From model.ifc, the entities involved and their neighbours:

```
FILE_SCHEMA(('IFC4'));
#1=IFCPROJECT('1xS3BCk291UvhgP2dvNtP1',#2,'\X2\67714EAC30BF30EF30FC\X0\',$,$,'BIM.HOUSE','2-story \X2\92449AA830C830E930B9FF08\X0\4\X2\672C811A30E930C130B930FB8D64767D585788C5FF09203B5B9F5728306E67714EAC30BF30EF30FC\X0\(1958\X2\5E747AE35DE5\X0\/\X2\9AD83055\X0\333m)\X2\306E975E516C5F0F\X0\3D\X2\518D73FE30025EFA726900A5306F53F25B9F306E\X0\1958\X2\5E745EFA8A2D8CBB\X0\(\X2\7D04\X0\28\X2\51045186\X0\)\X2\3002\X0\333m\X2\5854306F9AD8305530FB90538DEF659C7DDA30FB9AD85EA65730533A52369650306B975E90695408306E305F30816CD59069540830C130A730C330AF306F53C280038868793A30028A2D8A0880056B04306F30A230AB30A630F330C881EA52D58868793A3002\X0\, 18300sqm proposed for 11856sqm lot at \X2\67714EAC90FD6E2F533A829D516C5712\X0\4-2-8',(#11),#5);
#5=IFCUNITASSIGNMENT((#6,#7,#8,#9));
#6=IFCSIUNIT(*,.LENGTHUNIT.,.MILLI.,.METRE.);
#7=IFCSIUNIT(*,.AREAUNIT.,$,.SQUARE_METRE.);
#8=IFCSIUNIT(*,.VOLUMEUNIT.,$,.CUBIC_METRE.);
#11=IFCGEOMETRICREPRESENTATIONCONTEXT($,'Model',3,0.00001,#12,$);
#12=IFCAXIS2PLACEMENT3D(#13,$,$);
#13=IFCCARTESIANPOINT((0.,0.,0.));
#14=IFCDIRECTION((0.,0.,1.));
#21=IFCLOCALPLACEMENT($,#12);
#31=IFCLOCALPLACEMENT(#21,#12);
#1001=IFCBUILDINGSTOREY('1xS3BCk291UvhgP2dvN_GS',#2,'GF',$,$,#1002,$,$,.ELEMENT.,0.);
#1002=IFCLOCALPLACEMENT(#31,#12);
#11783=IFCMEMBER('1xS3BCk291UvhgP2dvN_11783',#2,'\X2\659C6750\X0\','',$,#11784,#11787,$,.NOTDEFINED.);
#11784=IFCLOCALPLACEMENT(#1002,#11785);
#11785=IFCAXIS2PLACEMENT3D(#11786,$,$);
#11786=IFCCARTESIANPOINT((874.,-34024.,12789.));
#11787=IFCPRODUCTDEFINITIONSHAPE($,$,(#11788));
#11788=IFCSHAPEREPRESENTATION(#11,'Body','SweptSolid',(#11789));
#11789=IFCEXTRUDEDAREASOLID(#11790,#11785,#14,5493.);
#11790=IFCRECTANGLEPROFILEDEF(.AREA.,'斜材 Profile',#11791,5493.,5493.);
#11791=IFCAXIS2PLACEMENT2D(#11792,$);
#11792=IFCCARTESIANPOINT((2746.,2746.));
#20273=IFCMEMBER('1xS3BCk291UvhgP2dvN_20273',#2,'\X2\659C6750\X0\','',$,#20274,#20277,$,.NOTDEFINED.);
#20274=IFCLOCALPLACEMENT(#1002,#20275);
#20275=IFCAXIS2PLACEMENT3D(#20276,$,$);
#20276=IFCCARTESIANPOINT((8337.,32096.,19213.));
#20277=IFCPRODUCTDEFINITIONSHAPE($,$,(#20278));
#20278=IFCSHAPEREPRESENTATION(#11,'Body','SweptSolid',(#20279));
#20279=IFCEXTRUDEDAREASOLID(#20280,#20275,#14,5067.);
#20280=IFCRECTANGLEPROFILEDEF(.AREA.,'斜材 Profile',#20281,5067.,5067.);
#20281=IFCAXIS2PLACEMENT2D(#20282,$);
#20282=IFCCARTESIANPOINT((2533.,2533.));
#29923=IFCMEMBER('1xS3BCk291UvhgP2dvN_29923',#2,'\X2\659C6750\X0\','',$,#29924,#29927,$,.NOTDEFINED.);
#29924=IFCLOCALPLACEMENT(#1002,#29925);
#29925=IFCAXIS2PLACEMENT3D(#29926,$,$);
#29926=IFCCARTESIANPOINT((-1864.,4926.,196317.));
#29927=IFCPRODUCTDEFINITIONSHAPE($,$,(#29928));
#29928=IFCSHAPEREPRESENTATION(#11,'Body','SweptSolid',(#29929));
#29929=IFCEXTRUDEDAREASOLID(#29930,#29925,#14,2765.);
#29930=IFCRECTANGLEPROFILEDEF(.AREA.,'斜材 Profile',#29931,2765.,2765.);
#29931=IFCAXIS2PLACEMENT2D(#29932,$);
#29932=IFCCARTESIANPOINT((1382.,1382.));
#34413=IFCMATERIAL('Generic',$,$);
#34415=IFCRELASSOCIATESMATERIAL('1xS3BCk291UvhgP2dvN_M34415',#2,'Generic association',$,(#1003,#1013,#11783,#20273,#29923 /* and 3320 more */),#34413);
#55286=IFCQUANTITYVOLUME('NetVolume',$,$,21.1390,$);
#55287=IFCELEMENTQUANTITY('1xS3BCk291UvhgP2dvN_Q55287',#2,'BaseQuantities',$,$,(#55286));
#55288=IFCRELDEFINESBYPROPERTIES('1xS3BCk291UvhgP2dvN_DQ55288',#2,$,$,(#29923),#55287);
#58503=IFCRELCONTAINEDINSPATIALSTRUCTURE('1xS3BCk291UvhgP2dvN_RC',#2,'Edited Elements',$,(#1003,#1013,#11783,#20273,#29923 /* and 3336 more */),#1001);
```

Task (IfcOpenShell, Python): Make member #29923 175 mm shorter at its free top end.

```python
import ifcopenshell
import ifcopenshell.api.pset
import ifcopenshell.util.element

model = ifcopenshell.open("model.ifc")

member = model.by_guid("1xS3BCk291UvhgP2dvN_29923")
change = -175.0

# The extrusion runs towards the end named, so only its depth changes.
body = next(r for r in member.Representation.Representations if r.RepresentationIdentifier == "Body")
solid = body.Items[0]
old_length = solid.Depth
solid.Depth += change

# Update the stored length and volume.
qto = model.by_id(ifcopenshell.util.element.get_pset(member, "BaseQuantities", should_inherit=False)["id"])
ifcopenshell.api.pset.edit_qto(model, qto=qto, properties={
    "NetVolume": ifcopenshell.util.element.get_pset(member, "BaseQuantities", "NetVolume") * solid.Depth / old_length,
})

print(f"length {old_length:g} -> {solid.Depth:g}")

model.write("model_updated.ifc")
```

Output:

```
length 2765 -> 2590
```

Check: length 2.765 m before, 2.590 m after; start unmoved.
